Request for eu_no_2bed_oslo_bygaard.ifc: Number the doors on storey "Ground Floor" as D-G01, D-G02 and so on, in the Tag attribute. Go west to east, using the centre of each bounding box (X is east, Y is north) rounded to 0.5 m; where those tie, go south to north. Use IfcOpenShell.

First a look at what the model holds.

```python
import ifcopenshell
import ifcopenshell.util.element
import ifcopenshell.util.placement

model = ifcopenshell.open("eu_no_2bed_oslo_bygaard.ifc")
print(model.schema)
storey = next(s for s in model.by_type("IfcBuildingStorey") if s.Name == "Ground Floor")
doors = [e for e in ifcopenshell.util.element.get_decomposition(storey) if e.is_a("IfcDoor")]
for e in sorted(doors, key=lambda e: e.id()):
    origin = ifcopenshell.util.placement.get_local_placement(e.ObjectPlacement)[:3, 3]
    print(e.id(), e.Tag, e.Name, origin.round(2) + 0.0, sep=" | ")
```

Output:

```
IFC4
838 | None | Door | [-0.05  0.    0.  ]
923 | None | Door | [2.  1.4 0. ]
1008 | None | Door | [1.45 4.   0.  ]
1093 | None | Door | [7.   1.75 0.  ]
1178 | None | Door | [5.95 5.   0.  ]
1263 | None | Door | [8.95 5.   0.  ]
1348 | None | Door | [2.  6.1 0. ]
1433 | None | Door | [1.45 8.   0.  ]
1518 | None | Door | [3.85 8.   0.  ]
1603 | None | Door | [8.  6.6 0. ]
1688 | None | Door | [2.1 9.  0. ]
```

```python
import ifcopenshell
import ifcopenshell.geom
import ifcopenshell.util.element
import ifcopenshell.util.shape

model = ifcopenshell.open("eu_no_2bed_oslo_bygaard.ifc")
settings = ifcopenshell.geom.settings()
settings.set("use-world-coords", True)


def centre(element):
    shape = ifcopenshell.geom.create_shape(settings, element)
    return ifcopenshell.util.shape.get_bbox_centroid(shape.geometry)


storey = next(s for s in model.by_type("IfcBuildingStorey") if s.Name == "Ground Floor")
doors = [e for e in ifcopenshell.util.element.get_decomposition(storey) if e.is_a("IfcDoor")]

# Insertion points can sit at a corner or the storey origin, so sort by the geometry (in metres).
centres = {e: centre(e) for e in doors}
doors.sort(key=lambda e: (round(centres[e][0] / 0.5), centres[e][1]))

for i, e in enumerate(doors, start=1):
    number = f"D-G{i:02d}"
    e.Tag = number
    print(e.id(), number)

model.write("eu_no_2bed_oslo_bygaard_edited.ifc")
```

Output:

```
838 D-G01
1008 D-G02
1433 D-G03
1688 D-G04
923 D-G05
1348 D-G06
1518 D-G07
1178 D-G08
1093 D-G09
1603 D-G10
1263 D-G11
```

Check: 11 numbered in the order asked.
